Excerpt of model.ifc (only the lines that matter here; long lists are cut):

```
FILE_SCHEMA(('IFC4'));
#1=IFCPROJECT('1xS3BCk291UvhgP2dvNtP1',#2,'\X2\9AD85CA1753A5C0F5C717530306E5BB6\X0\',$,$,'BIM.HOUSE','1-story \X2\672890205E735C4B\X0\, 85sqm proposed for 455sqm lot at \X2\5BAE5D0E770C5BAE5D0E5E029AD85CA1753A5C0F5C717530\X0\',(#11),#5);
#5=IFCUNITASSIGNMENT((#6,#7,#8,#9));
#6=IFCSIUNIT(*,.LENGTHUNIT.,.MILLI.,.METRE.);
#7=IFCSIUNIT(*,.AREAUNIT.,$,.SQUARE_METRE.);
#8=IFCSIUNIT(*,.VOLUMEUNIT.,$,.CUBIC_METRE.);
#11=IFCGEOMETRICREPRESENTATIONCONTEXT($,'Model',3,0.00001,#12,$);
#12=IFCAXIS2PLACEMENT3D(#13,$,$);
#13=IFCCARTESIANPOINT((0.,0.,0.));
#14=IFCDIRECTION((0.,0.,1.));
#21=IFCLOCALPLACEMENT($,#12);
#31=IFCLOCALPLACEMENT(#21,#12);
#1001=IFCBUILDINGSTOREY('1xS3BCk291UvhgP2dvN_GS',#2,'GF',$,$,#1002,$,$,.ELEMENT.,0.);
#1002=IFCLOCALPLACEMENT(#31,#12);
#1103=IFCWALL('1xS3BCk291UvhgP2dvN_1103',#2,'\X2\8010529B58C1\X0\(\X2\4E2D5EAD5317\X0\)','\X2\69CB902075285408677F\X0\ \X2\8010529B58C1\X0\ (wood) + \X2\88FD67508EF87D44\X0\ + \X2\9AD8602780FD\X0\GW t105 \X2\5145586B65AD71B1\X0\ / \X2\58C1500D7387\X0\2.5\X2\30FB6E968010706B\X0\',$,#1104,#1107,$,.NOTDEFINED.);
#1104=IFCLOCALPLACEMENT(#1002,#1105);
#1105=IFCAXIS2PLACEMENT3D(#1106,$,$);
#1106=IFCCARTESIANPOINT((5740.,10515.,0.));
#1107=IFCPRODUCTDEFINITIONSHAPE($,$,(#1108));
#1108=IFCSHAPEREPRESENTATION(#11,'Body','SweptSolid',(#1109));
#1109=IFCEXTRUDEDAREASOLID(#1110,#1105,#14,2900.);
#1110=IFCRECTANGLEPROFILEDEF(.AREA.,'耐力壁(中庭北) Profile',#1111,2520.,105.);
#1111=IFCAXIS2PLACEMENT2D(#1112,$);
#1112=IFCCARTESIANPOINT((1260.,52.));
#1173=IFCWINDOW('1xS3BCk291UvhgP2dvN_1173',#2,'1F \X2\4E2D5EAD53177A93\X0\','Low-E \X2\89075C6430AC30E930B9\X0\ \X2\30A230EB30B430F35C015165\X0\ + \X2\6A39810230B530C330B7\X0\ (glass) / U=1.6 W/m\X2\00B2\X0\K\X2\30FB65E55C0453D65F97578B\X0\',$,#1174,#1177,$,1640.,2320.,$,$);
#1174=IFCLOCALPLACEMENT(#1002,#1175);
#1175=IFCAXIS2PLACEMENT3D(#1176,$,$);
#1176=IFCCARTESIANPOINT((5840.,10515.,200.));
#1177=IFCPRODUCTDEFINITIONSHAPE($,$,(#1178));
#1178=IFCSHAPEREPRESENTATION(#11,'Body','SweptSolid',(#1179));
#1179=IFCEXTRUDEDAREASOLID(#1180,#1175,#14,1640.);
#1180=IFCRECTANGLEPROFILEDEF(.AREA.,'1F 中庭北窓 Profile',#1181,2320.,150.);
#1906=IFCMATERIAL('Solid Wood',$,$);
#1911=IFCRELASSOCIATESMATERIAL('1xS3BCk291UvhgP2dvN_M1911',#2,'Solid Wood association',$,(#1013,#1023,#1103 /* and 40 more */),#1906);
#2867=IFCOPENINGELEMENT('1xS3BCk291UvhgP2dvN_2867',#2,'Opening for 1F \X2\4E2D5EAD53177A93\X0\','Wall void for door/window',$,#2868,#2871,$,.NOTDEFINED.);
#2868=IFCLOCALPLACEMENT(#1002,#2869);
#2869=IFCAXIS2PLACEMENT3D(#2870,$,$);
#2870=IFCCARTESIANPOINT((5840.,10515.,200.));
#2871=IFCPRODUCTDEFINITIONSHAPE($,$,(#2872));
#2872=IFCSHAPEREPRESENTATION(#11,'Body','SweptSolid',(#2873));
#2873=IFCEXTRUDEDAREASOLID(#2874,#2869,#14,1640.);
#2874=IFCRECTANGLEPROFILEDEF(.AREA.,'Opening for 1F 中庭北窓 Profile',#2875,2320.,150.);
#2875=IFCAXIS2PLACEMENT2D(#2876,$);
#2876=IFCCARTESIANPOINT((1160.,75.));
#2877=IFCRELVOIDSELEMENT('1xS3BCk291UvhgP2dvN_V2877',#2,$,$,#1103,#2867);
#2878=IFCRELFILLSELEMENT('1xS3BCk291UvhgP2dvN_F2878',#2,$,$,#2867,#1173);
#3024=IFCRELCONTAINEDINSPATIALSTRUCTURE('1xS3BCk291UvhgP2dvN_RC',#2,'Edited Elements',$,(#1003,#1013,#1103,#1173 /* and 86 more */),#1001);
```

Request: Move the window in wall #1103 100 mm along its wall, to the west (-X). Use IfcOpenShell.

```python
import ifcopenshell
import ifcopenshell.api.geometry
import ifcopenshell.util.placement
import ifcopenshell.util.unit

model = ifcopenshell.open("model.ifc")
unit_scale = ifcopenshell.util.unit.calculate_unit_scale(model)

window = model.by_guid("1xS3BCk291UvhgP2dvN_1173")
opening = window.FillsVoids[0].RelatingOpeningElement
wall = opening.VoidsElements[0].RelatingBuildingElement

wall_matrix = ifcopenshell.util.placement.get_local_placement(wall.ObjectPlacement)
shift = wall_matrix[:3, 0] * -0.1 / unit_scale
before = ifcopenshell.util.placement.get_local_placement(window.ObjectPlacement)[:3, 3].copy()

# The window is not placed relative to its opening, so move both.
for product in (opening, window):
    matrix = ifcopenshell.util.placement.get_local_placement(product.ObjectPlacement)
    matrix[:3, 3] += shift
    ifcopenshell.api.geometry.edit_object_placement(model, product=product, matrix=matrix, is_si=False)

after = ifcopenshell.util.placement.get_local_placement(window.ObjectPlacement)[:3, 3]
print("window moved by", (after - before).round(3) + 0.0)

model.write("model-out.ifc")
```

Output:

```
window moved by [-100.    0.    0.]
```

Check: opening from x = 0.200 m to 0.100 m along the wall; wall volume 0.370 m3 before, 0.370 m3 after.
